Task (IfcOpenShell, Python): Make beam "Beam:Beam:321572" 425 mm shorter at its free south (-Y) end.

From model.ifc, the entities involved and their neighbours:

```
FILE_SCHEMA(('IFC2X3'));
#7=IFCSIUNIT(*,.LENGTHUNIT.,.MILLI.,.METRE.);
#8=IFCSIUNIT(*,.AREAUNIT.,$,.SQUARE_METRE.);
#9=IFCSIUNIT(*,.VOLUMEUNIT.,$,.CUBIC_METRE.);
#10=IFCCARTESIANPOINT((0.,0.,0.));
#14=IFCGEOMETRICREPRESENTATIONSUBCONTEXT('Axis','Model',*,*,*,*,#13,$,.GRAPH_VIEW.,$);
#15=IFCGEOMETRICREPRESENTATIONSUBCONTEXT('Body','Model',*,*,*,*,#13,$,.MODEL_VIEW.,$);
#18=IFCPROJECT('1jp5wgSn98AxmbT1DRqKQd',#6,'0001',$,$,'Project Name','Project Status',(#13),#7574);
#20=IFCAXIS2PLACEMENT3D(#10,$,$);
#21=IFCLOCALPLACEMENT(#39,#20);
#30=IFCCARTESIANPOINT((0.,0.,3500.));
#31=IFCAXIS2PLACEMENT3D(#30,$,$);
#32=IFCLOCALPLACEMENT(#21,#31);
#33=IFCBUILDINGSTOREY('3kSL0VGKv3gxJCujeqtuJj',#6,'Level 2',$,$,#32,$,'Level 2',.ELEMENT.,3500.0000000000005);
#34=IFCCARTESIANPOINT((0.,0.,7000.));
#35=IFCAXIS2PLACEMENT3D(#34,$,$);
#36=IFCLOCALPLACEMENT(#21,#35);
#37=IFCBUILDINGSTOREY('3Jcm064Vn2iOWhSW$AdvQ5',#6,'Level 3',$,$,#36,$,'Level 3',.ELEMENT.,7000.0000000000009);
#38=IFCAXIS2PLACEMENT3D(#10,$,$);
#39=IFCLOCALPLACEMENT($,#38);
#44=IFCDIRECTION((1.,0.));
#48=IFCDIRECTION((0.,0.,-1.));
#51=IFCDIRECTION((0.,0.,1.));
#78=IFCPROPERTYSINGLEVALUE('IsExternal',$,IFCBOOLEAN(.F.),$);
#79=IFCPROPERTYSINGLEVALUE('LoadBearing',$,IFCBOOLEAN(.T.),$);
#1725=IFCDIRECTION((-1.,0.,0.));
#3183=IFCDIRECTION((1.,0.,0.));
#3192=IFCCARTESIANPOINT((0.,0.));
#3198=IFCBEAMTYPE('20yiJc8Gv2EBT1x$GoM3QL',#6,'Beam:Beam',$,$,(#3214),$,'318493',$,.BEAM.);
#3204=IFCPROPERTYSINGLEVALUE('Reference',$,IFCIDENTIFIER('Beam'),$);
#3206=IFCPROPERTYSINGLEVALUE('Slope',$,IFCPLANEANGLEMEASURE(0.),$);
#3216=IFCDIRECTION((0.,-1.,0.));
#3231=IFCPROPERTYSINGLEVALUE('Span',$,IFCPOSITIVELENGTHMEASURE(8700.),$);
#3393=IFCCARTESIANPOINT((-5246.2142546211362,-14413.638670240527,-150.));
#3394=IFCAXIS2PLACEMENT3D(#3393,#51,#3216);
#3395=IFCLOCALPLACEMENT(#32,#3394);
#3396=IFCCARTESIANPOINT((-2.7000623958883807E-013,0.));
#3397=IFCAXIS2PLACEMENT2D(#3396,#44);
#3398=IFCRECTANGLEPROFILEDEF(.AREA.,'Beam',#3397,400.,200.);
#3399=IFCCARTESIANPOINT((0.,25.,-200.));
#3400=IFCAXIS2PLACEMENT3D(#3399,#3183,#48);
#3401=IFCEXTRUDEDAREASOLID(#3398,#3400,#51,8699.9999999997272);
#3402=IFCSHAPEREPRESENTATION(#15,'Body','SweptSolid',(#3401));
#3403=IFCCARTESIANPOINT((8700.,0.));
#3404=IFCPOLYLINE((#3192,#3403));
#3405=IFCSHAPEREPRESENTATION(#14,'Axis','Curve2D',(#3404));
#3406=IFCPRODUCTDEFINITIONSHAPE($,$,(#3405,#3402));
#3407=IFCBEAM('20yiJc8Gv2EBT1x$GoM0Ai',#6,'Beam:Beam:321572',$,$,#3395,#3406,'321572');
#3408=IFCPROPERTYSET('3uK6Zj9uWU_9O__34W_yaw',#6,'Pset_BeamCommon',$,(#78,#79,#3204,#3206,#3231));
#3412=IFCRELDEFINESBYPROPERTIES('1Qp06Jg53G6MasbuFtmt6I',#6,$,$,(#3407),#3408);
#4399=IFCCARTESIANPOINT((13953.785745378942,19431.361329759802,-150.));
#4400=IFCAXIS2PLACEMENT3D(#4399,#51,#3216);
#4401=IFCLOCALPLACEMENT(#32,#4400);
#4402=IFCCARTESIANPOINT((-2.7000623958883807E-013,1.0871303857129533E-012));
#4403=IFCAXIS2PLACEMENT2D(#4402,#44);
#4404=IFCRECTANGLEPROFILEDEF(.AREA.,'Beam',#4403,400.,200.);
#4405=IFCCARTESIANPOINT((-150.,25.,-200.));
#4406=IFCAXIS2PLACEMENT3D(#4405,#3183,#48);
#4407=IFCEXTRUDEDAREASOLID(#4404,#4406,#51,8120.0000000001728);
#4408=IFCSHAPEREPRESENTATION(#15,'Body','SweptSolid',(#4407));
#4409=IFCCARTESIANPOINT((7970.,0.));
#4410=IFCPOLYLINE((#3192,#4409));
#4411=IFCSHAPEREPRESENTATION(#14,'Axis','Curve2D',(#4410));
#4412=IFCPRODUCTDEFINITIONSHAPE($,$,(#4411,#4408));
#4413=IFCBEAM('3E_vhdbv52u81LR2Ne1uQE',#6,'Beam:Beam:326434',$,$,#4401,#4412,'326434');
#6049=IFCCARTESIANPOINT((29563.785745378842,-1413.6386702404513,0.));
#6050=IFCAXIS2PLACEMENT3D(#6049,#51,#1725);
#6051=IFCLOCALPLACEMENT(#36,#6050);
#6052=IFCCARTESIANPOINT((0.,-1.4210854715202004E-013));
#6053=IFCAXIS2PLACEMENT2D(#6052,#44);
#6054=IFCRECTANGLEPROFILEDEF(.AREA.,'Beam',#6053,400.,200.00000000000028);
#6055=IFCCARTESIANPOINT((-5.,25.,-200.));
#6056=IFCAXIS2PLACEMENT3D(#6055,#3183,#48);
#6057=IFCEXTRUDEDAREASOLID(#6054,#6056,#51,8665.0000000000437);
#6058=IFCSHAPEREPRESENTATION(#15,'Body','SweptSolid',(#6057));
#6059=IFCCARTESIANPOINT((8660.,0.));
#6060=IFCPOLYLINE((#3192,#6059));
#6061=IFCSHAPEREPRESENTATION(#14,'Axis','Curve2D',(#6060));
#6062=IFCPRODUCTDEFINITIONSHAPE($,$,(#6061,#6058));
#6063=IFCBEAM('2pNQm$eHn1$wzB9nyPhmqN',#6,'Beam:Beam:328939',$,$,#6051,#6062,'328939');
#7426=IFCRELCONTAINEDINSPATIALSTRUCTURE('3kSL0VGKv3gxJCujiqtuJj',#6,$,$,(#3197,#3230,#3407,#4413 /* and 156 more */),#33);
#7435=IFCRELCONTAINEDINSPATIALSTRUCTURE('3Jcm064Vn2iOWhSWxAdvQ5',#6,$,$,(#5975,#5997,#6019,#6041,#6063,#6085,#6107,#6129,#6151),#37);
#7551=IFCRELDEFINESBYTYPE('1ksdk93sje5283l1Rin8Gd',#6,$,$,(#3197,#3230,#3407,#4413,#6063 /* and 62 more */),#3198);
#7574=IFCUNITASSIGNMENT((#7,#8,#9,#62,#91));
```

```python
import numpy as np
import ifcopenshell
import ifcopenshell.api.pset
import ifcopenshell.util.element
import ifcopenshell.util.representation

model = ifcopenshell.open("model.ifc")

member = model.by_id(3407)
change = -425.0

# The extrusion runs towards the end named, so only its depth changes.
body = ifcopenshell.util.representation.get_representation(member, "Model", "Body")
solid = body.Items[0]
old_length = solid.Depth
solid.Depth += change

# Move the axis end point with it.
axis = next(r for r in member.Representation.Representations if r.RepresentationIdentifier == "Axis").Items[0]
start, end = (np.array(p.Coordinates) for p in axis.Points)
end = end + (end - start) / np.linalg.norm(end - start) * change
point = model.createIfcCartesianPoint(end.tolist())
axis.Points = [axis.Points[0], point]

# Update the stored length and volume.
pset = model.by_id(ifcopenshell.util.element.get_pset(member, "Pset_BeamCommon", should_inherit=False)["id"])
ifcopenshell.api.pset.edit_pset(model, pset=pset, properties={
    "Span": model.create_entity("IfcPositiveLengthMeasure", solid.Depth),
})

print(f"length {old_length:g} -> {solid.Depth:g}")

model.write("model_rev.ifc")
```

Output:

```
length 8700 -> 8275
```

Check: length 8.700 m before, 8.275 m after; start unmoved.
